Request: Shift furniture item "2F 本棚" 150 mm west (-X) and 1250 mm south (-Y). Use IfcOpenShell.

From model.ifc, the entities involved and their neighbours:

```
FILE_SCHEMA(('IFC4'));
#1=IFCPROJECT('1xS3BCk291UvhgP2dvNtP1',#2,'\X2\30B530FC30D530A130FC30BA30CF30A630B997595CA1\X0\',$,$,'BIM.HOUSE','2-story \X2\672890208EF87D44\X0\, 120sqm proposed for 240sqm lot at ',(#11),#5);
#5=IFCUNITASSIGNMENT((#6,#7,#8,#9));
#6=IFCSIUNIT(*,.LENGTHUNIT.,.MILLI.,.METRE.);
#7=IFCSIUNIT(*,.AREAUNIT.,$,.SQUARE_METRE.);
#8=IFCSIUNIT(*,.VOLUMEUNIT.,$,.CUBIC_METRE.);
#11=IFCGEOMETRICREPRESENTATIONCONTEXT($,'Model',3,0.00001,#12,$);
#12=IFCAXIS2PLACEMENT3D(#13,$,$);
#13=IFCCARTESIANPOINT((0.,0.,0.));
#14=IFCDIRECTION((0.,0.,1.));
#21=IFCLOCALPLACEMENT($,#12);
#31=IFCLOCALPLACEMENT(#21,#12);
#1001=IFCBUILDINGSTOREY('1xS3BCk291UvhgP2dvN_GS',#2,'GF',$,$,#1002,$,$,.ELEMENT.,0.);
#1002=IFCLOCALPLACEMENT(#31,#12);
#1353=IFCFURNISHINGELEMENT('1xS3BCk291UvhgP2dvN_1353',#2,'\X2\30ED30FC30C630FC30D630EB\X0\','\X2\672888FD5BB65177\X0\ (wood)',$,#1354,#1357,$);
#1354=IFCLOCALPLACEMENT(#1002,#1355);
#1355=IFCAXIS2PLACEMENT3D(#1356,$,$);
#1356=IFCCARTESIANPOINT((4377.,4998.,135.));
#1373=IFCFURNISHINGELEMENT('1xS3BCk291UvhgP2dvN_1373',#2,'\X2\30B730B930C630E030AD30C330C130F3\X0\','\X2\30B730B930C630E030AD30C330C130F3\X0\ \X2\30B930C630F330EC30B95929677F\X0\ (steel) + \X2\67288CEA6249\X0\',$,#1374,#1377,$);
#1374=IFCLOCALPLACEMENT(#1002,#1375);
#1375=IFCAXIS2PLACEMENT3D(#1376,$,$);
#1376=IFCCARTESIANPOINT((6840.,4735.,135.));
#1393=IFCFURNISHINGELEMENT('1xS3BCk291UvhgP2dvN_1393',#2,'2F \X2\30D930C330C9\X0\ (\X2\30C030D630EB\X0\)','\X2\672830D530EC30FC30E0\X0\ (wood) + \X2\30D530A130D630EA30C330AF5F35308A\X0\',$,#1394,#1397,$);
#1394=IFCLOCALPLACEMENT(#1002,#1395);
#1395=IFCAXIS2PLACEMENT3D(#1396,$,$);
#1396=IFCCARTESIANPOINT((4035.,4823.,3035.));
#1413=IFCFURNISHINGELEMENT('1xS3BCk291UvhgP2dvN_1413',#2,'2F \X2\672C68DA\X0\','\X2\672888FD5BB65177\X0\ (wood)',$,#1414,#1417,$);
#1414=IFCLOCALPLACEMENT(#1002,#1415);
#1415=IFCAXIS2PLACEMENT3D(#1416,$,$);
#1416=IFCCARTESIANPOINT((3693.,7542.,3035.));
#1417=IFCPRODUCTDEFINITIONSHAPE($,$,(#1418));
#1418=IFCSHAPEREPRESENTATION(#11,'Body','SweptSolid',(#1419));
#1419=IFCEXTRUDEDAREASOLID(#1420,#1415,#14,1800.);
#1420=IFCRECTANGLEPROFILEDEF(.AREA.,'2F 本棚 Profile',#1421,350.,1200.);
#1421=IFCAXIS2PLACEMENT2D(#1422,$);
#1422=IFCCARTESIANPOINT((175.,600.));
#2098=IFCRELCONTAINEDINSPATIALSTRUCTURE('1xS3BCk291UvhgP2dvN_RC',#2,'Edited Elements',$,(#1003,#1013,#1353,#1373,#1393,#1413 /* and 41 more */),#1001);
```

```python
import ifcopenshell
import ifcopenshell.api.geometry
import ifcopenshell.util.placement
import ifcopenshell.util.unit

model = ifcopenshell.open("model.ifc")
unit_scale = ifcopenshell.util.unit.calculate_unit_scale(model)

item = model.by_guid("1xS3BCk291UvhgP2dvN_1413")
matrix = ifcopenshell.util.placement.get_local_placement(item.ObjectPlacement)
matrix[0, 3] -= 0.15 / unit_scale
matrix[1, 3] -= 1.25 / unit_scale
ifcopenshell.api.geometry.edit_object_placement(model, product=item, matrix=matrix, is_si=False)

print(ifcopenshell.util.placement.get_local_placement(item.ObjectPlacement).round(3) + 0.0)

model.write("model_edited.ifc")
```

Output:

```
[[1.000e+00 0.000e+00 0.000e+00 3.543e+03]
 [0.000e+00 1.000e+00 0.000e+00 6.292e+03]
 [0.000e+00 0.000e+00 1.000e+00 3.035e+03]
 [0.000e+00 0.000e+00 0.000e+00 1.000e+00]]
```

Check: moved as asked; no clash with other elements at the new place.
